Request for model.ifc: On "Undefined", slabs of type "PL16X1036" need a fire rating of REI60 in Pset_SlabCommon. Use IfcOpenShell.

First a look at what the model holds.

```python
import ifcopenshell
import ifcopenshell.util.element

model = ifcopenshell.open("model.ifc")
print(model.schema)
storey = next(s for s in model.by_type("IfcBuildingStorey") if s.Name == "Undefined")
slabs = [e for e in ifcopenshell.util.element.get_decomposition(storey) if e.is_a("IfcSlab")]
seen = {}
for e in slabs:
    element_type = ifcopenshell.util.element.get_type(e)
    key = (element_type.Name if element_type != e and element_type else None, ifcopenshell.util.element.get_pset(e, "Pset_SlabCommon", "FireRating"))
    seen[key] = seen.get(key, 0) + 1
for (name, value), count in sorted(seen.items(), key=str):
    print(count, "x", name, "|", value)
```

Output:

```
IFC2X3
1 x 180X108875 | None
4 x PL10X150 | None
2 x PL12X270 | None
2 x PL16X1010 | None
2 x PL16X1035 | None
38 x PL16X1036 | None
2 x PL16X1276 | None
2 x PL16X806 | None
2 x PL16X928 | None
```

```python
import ifcopenshell
import ifcopenshell.api.pset
import ifcopenshell.util.element

model = ifcopenshell.open("model.ifc")

storey = next(s for s in model.by_type("IfcBuildingStorey") if s.Name == "Undefined")
slabs = [e for e in ifcopenshell.util.element.get_decomposition(storey) if e.is_a("IfcSlab")]

count = 0
for e in slabs:
    element_type = ifcopenshell.util.element.get_type(e)
    if element_type in (None, e) or element_type.Name != "PL16X1036":
        continue
    # add_pset returns the element's existing set when there is one.
    pset = ifcopenshell.api.pset.add_pset(model, product=e, name="Pset_SlabCommon")
    ifcopenshell.api.pset.edit_pset(model, pset=pset, properties={"FireRating": "REI60"})
    count += 1

print(count, "slabs updated")

model.write("model-out.ifc")
```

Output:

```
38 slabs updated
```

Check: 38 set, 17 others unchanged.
